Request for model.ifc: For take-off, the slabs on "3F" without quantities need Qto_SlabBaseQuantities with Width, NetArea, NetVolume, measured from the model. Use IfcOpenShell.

First a look at what the model holds.

```python
import ifcopenshell
import ifcopenshell.util.element
import ifcopenshell.util.unit

model = ifcopenshell.open("model.ifc")
print(model.schema)
for unit_type in ("LENGTHUNIT", "AREAUNIT", "VOLUMEUNIT"):
    print(unit_type, ifcopenshell.util.unit.calculate_unit_scale(model, unit_type))
storey = next(s for s in model.by_type("IfcBuildingStorey") if s.Name == "3F")
slabs = [e for e in ifcopenshell.util.element.get_decomposition(storey) if e.is_a("IfcSlab")]
for e in sorted(slabs, key=lambda e: e.id()):
    print(e.id(), e.is_a(), e.Name, list(ifcopenshell.util.element.get_psets(e, qtos_only=True)), sep=" | ")
```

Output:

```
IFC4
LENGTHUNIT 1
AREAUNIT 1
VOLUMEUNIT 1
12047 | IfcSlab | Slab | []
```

```python
import ifcopenshell
import ifcopenshell.api.pset
import ifcopenshell.geom
import ifcopenshell.util.element
import ifcopenshell.util.shape
import ifcopenshell.util.unit

model = ifcopenshell.open("model.ifc")
unit_scale = ifcopenshell.util.unit.calculate_unit_scale(model)
area_scale = ifcopenshell.util.unit.calculate_unit_scale(model, "AREAUNIT")
volume_scale = ifcopenshell.util.unit.calculate_unit_scale(model, "VOLUMEUNIT")
settings = ifcopenshell.geom.settings()

storey = next(s for s in model.by_type("IfcBuildingStorey") if s.Name == "3F")
slabs = [e for e in ifcopenshell.util.element.get_decomposition(storey) if e.is_a("IfcSlab")]

for e in sorted(slabs, key=lambda e: e.id()):
    if ifcopenshell.util.element.get_psets(e, qtos_only=True, should_inherit=False):
        continue
    # Geometry comes back in metres, in the element's own axes.
    shape = ifcopenshell.geom.create_shape(settings, e)
    values = {
        "Width": ifcopenshell.util.shape.get_z(shape.geometry) / unit_scale,
        "NetArea": ifcopenshell.util.shape.get_footprint_area(shape.geometry) / area_scale,
        "NetVolume": ifcopenshell.util.shape.get_volume(shape.geometry) / volume_scale,
    }
    qto = ifcopenshell.api.pset.add_qto(model, product=e, name="Qto_SlabBaseQuantities")
    ifcopenshell.api.pset.edit_qto(model, qto=qto, properties=values)
    print(e.id(), {k: round(v, 3) for k, v in values.items()})

model.write("model_edited.ifc")
```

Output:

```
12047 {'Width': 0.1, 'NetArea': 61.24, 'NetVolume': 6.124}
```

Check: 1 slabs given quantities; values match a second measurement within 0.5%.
